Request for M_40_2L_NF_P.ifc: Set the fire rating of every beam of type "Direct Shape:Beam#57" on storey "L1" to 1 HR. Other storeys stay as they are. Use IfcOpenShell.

First a look at what the model holds.

```python
import ifcopenshell
import ifcopenshell.util.element

model = ifcopenshell.open("M_40_2L_NF_P.ifc")
print(model.schema)
storey = next(s for s in model.by_type("IfcBuildingStorey") if s.Name == "L1")
beams = [e for e in ifcopenshell.util.element.get_decomposition(storey) if e.is_a("IfcBeam")]
seen = {}
for e in beams:
    element_type = ifcopenshell.util.element.get_type(e)
    key = (element_type.Name if element_type != e and element_type else None, ifcopenshell.util.element.get_pset(e, "Pset_BeamCommon", "FireRating"))
    seen[key] = seen.get(key, 0) + 1
for (name, value), count in sorted(seen.items(), key=str):
    print(count, "x", name, "|", value)
```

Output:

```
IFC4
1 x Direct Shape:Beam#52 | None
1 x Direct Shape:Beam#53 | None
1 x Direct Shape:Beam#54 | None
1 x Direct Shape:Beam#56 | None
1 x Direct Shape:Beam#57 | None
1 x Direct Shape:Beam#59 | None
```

```python
import ifcopenshell
import ifcopenshell.api.pset
import ifcopenshell.util.element

model = ifcopenshell.open("M_40_2L_NF_P.ifc")

storey = next(s for s in model.by_type("IfcBuildingStorey") if s.Name == "L1")
beams = [e for e in ifcopenshell.util.element.get_decomposition(storey) if e.is_a("IfcBeam")]

count = 0
for e in beams:
    element_type = ifcopenshell.util.element.get_type(e)
    if element_type in (None, e) or element_type.Name != "Direct Shape:Beam#57":
        continue
    # add_pset returns the element's existing set when there is one.
    pset = ifcopenshell.api.pset.add_pset(model, product=e, name="Pset_BeamCommon")
    ifcopenshell.api.pset.edit_pset(model, pset=pset, properties={"FireRating": "1 HR"})
    count += 1

print(count, "beams updated")

model.write("M_40_2L_NF_P_edited.ifc")
```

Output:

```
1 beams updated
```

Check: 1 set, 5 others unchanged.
